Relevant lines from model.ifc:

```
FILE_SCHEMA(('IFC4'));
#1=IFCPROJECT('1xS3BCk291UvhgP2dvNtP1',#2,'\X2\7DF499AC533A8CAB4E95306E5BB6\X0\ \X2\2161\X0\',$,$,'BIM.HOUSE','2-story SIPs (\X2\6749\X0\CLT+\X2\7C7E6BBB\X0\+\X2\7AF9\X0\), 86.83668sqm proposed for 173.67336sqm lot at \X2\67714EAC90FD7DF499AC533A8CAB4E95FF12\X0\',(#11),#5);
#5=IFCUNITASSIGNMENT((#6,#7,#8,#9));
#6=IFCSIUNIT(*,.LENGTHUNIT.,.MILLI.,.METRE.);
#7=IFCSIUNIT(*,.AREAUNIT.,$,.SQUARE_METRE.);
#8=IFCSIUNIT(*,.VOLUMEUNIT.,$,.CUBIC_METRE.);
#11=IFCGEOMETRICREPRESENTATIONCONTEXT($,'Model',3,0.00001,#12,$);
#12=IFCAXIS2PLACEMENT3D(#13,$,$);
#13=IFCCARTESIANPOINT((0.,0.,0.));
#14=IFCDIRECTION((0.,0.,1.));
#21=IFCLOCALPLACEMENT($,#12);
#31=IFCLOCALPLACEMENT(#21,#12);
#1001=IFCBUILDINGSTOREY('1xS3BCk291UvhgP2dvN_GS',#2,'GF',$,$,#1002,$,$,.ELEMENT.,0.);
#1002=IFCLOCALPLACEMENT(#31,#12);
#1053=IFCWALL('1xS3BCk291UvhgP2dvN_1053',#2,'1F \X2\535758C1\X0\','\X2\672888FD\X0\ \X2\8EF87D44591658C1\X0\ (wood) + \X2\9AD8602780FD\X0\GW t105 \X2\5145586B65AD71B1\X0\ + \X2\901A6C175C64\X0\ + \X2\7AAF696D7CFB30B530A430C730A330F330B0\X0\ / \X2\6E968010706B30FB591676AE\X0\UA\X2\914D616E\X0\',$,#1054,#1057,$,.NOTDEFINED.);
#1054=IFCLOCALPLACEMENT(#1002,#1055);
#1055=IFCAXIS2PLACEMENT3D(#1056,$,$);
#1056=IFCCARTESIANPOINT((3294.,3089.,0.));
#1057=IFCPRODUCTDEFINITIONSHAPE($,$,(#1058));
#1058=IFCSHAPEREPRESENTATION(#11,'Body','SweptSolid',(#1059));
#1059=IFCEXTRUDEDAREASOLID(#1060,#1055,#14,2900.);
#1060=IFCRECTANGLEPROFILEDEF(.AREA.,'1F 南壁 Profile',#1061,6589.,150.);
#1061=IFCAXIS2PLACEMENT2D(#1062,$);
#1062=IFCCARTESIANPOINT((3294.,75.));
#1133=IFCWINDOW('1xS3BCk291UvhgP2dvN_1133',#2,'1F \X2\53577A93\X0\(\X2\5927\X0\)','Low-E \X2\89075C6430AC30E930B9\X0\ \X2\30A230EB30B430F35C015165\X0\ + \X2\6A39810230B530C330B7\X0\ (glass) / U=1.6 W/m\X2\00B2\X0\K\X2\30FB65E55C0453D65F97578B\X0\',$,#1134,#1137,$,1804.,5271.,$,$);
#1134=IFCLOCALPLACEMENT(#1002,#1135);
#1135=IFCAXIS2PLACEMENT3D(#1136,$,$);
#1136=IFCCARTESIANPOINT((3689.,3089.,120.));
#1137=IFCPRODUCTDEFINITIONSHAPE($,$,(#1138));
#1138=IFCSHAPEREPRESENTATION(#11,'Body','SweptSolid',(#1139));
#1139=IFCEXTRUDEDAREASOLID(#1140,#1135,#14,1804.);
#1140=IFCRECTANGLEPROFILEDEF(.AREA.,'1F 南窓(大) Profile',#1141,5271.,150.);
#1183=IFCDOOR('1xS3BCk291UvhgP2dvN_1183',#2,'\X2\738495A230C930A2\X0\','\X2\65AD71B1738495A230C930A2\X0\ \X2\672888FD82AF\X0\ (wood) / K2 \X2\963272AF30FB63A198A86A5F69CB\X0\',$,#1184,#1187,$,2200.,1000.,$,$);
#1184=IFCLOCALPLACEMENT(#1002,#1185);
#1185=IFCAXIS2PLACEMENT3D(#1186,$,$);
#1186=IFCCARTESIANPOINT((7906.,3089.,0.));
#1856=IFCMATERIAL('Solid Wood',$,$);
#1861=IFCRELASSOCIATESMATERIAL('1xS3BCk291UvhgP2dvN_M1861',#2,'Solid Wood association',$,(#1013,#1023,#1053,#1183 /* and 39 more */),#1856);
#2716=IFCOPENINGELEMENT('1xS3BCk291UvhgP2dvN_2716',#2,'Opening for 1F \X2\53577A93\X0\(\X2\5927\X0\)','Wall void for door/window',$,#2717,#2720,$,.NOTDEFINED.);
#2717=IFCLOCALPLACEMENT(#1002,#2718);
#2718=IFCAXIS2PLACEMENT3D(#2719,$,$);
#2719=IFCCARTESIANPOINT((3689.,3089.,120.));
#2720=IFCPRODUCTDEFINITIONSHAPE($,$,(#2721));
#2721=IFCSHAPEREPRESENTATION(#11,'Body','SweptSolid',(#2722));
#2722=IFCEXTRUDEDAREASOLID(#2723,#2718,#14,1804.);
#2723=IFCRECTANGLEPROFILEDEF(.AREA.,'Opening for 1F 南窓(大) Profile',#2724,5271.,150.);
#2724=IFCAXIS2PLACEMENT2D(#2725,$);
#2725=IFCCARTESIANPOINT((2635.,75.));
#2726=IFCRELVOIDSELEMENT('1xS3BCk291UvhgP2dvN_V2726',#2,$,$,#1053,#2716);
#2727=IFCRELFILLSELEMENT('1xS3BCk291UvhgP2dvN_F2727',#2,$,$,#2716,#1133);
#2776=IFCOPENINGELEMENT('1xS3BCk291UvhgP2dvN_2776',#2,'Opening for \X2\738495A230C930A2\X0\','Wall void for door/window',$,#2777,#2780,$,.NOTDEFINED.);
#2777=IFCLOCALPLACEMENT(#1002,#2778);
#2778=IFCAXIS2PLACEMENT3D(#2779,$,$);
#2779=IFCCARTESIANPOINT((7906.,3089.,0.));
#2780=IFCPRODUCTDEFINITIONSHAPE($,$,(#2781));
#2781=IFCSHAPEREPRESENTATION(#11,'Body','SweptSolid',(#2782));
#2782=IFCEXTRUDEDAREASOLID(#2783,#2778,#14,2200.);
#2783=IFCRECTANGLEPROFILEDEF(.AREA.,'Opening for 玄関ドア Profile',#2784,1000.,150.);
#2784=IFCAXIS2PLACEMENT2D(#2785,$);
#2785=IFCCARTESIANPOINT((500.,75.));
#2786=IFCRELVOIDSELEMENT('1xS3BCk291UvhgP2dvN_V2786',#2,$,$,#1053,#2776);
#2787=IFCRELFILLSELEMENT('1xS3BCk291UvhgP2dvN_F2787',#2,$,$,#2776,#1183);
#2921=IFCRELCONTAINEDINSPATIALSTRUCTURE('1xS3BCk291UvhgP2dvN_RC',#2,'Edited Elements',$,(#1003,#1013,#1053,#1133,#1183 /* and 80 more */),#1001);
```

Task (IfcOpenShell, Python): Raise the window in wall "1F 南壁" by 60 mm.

```python
import numpy as np
import ifcopenshell
import ifcopenshell.api.geometry
import ifcopenshell.util.placement
import ifcopenshell.util.unit

model = ifcopenshell.open("model.ifc")
unit_scale = ifcopenshell.util.unit.calculate_unit_scale(model)

window = model.by_guid("1xS3BCk291UvhgP2dvN_1133")
opening = window.FillsVoids[0].RelatingOpeningElement
dz = 0.06 / unit_scale

shift = np.array([0.0, 0.0, dz])
# The window is not placed relative to its opening, so move both.
for product in (opening, window):
    matrix = ifcopenshell.util.placement.get_local_placement(product.ObjectPlacement)
    matrix[:3, 3] += shift
    ifcopenshell.api.geometry.edit_object_placement(model, product=product, matrix=matrix, is_si=False)

print(f"moved by {dz * unit_scale:+.3f} m")

model.write("model_rev.ifc")
```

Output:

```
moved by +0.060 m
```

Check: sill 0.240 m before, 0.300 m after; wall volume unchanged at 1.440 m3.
